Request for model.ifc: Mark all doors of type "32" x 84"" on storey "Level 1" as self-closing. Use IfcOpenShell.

First a look at what the model holds.

```python
import ifcopenshell
import ifcopenshell.util.element

model = ifcopenshell.open("model.ifc")
print(model.schema)
storey = next(s for s in model.by_type("IfcBuildingStorey") if s.Name == "Level 1")
doors = [e for e in ifcopenshell.util.element.get_decomposition(storey) if e.is_a("IfcDoor")]
seen = {}
for e in doors:
    element_type = ifcopenshell.util.element.get_type(e)
    key = (element_type.Name if element_type != e and element_type else None, ifcopenshell.util.element.get_pset(e, "Pset_DoorCommon", "SelfClosing"))
    seen[key] = seen.get(key, 0) + 1
for (name, value), count in sorted(seen.items(), key=str):
    print(count, "x", name, "|", value)
```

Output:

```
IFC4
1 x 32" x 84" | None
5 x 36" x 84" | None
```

```python
import ifcopenshell
import ifcopenshell.api.pset
import ifcopenshell.util.element

model = ifcopenshell.open("model.ifc")

storey = next(s for s in model.by_type("IfcBuildingStorey") if s.Name == "Level 1")
doors = [e for e in ifcopenshell.util.element.get_decomposition(storey) if e.is_a("IfcDoor")]

count = 0
for e in doors:
    element_type = ifcopenshell.util.element.get_type(e)
    if element_type in (None, e) or element_type.Name != '32" x 84"':
        continue
    # add_pset returns the element's existing set when there is one.
    pset = ifcopenshell.api.pset.add_pset(model, product=e, name="Pset_DoorCommon")
    ifcopenshell.api.pset.edit_pset(model, pset=pset, properties={"SelfClosing": True})
    count += 1

print(count, "doors updated")

model.write("model_rev.ifc")
```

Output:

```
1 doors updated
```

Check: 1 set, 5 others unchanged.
